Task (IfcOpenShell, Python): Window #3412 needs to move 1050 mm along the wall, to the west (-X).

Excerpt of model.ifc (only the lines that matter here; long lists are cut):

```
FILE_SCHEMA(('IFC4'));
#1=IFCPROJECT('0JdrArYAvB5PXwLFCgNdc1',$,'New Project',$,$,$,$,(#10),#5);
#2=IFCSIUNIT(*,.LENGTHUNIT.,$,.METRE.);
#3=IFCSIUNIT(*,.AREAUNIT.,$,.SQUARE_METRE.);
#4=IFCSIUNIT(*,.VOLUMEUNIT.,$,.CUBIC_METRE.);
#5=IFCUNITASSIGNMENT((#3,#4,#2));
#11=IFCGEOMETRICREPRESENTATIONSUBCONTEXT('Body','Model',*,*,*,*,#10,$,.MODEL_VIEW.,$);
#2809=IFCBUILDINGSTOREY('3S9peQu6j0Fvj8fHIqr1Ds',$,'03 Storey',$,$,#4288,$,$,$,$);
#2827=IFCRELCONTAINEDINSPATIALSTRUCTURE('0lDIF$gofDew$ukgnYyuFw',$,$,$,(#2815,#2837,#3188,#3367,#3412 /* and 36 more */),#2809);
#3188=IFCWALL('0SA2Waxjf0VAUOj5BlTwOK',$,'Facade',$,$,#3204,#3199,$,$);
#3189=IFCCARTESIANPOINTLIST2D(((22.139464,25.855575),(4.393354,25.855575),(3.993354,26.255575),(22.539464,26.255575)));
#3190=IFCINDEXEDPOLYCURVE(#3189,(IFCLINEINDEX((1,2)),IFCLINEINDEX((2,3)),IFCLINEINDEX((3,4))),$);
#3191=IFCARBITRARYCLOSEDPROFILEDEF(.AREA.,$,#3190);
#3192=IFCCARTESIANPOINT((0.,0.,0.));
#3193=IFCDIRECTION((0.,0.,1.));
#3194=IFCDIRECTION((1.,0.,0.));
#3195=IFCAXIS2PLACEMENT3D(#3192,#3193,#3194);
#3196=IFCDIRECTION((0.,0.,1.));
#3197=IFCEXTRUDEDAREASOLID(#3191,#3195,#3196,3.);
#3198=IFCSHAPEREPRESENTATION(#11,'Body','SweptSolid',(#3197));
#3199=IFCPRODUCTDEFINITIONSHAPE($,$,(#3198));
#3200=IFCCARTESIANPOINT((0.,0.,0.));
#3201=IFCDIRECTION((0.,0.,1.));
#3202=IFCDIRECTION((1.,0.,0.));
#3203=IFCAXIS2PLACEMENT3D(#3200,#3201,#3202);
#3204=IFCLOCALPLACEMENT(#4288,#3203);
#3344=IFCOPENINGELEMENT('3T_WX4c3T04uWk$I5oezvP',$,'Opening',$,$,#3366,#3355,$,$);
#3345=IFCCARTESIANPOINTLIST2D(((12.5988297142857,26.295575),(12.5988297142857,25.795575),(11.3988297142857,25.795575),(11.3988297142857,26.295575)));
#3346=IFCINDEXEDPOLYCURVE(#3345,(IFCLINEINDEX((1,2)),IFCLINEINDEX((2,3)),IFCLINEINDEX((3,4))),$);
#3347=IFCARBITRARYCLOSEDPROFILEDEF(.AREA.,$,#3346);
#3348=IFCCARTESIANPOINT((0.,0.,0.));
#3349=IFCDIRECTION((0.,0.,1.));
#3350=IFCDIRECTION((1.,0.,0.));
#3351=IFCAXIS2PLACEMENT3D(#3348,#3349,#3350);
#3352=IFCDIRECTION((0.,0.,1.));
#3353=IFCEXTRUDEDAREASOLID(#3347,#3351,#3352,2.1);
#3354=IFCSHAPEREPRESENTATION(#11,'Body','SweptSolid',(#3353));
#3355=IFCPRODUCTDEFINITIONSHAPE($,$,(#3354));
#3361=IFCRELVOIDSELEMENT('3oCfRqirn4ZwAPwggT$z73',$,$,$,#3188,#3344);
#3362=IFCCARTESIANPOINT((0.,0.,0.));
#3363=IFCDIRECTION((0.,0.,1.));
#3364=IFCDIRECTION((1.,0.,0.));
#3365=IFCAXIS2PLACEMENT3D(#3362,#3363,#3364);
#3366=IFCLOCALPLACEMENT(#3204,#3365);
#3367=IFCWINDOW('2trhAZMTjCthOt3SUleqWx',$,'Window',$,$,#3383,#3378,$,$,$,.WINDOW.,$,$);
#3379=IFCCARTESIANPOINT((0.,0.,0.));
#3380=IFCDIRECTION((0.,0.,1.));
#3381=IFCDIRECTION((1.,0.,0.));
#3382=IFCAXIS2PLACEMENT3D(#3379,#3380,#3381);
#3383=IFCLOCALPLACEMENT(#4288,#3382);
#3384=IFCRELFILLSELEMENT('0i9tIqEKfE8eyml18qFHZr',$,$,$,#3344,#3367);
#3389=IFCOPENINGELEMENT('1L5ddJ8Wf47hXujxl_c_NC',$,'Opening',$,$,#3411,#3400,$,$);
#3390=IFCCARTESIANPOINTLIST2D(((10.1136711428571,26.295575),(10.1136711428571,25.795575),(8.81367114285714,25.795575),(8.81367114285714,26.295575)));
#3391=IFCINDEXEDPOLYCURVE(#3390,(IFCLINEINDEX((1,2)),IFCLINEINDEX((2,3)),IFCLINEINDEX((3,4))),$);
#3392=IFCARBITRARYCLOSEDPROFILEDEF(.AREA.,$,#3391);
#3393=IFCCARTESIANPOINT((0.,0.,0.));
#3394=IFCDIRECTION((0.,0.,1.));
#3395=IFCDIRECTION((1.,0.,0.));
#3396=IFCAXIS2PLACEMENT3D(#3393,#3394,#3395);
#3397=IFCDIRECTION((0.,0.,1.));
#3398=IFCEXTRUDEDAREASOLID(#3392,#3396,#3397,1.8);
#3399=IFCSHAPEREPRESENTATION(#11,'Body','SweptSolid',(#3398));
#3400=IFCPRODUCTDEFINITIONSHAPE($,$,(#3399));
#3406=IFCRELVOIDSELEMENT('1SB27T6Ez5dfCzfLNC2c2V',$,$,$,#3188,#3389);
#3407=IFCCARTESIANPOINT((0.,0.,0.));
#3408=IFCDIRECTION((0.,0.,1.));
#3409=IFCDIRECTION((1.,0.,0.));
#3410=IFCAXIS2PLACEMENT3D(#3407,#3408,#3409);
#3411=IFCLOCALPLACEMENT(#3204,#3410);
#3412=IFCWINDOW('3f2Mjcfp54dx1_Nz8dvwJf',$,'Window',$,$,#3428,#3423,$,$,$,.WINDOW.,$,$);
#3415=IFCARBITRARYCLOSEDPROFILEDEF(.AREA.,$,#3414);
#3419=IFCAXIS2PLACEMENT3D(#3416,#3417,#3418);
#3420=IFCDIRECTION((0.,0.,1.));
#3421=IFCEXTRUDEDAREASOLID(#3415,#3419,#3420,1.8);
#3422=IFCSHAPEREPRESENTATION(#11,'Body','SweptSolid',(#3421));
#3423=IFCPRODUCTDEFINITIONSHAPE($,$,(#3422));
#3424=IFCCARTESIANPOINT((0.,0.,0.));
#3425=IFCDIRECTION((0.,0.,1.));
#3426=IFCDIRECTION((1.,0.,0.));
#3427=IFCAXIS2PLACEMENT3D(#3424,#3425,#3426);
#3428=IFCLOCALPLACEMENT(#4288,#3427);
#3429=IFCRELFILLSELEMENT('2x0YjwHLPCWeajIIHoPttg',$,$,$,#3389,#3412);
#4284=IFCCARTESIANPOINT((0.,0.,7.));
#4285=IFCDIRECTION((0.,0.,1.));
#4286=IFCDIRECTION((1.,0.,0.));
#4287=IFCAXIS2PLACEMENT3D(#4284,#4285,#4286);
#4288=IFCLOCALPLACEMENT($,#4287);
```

```python
import ifcopenshell
import ifcopenshell.api.geometry
import ifcopenshell.util.placement
import ifcopenshell.util.unit

model = ifcopenshell.open("model.ifc")
unit_scale = ifcopenshell.util.unit.calculate_unit_scale(model)

window = model.by_id(3412)
opening = window.FillsVoids[0].RelatingOpeningElement
wall = opening.VoidsElements[0].RelatingBuildingElement

wall_matrix = ifcopenshell.util.placement.get_local_placement(wall.ObjectPlacement)
shift = wall_matrix[:3, 0] * -1.05 / unit_scale
before = ifcopenshell.util.placement.get_local_placement(window.ObjectPlacement)[:3, 3].copy()

# The window is not placed relative to its opening, so move both.
for product in (opening, window):
    matrix = ifcopenshell.util.placement.get_local_placement(product.ObjectPlacement)
    matrix[:3, 3] += shift
    ifcopenshell.api.geometry.edit_object_placement(model, product=product, matrix=matrix, is_si=False)

after = ifcopenshell.util.placement.get_local_placement(window.ObjectPlacement)[:3, 3]
print("window moved by", (after - before).round(3) + 0.0)

model.write("model_updated.ifc")
```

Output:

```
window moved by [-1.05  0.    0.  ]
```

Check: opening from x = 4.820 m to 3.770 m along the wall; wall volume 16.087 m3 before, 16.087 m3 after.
